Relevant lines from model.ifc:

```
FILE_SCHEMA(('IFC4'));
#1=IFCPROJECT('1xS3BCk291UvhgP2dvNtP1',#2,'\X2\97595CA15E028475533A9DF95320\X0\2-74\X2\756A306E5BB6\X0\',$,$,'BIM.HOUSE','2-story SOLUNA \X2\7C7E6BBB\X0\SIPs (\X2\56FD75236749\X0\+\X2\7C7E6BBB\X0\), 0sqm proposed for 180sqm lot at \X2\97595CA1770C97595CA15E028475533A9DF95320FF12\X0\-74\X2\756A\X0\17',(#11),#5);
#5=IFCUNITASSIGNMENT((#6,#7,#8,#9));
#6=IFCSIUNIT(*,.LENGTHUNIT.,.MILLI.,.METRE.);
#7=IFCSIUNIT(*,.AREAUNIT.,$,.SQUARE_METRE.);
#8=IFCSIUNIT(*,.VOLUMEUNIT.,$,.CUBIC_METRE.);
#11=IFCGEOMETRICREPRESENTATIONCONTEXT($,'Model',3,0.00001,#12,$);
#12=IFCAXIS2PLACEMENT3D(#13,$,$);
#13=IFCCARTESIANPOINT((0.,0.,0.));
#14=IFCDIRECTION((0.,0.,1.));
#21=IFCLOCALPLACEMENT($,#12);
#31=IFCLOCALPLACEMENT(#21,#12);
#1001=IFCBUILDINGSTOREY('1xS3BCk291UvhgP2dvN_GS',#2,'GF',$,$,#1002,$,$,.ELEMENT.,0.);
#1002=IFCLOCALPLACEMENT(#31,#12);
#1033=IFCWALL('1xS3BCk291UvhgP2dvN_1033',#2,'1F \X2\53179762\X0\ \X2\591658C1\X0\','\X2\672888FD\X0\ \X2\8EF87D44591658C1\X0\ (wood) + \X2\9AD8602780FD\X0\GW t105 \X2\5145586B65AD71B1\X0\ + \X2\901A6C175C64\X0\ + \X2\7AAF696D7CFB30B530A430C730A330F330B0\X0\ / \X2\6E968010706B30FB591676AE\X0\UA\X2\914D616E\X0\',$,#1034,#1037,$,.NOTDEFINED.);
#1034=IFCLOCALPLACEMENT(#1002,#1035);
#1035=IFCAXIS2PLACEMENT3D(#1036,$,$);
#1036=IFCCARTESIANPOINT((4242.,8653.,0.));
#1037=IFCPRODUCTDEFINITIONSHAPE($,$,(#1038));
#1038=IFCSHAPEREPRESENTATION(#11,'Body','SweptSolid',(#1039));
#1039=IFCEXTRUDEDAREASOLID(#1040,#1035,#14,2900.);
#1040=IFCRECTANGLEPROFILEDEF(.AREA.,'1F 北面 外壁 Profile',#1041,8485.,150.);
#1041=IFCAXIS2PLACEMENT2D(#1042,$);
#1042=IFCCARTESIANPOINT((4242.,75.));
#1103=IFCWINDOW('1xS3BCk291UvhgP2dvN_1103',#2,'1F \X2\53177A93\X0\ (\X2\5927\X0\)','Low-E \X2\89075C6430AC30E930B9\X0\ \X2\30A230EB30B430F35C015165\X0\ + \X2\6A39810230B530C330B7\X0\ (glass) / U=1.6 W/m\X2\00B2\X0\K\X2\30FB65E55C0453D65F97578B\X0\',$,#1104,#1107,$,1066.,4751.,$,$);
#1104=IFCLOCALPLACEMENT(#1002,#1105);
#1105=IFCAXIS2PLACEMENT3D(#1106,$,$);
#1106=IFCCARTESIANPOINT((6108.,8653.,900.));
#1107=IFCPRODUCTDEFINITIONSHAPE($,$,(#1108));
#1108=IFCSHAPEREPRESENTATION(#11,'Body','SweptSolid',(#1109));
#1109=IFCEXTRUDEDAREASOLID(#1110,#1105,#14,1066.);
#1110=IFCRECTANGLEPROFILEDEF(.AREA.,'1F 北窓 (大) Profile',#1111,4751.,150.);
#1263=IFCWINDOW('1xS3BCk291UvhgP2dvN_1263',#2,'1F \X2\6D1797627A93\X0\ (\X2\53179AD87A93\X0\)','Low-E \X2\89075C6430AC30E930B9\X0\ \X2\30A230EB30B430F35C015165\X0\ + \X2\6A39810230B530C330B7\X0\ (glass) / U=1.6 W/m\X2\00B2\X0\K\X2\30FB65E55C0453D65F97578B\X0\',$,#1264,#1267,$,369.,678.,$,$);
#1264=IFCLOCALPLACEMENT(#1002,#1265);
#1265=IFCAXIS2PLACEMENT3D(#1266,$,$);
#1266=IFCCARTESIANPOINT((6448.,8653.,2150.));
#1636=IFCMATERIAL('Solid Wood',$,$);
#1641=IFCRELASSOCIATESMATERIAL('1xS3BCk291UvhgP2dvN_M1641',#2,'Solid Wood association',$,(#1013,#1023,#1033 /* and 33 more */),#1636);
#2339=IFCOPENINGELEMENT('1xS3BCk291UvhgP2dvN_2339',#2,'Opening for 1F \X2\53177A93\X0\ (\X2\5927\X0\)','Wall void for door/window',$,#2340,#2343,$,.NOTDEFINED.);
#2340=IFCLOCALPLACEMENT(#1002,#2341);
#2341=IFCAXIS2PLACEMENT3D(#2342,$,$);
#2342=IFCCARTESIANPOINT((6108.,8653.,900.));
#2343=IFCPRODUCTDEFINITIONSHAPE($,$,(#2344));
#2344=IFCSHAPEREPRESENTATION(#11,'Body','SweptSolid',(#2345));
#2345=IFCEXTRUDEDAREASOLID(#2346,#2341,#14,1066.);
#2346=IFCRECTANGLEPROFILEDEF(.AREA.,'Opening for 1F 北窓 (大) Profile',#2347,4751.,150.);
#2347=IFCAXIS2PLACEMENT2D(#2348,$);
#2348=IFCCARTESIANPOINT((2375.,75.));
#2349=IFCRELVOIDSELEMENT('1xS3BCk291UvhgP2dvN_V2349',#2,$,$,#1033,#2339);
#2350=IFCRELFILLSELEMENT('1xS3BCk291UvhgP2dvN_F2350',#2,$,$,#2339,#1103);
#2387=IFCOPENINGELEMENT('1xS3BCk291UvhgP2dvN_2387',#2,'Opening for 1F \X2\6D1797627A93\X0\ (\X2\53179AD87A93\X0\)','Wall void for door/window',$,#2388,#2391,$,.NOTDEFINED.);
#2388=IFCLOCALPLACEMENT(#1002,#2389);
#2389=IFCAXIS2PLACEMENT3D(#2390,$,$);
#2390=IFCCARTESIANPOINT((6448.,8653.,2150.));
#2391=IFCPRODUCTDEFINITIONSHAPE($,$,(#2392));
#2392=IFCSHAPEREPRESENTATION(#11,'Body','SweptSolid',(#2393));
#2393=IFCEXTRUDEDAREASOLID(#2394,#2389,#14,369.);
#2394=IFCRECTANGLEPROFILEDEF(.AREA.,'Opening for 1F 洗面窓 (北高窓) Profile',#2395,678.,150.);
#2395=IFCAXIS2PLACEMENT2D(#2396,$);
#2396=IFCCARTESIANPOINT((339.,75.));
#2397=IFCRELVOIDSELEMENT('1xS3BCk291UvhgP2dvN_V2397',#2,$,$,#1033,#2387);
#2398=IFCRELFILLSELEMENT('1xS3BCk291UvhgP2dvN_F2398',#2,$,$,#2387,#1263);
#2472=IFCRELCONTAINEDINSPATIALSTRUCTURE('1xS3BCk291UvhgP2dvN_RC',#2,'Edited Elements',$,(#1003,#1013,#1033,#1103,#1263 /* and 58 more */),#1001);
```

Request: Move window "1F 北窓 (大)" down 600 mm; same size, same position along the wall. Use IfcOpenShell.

```python
import numpy as np
import ifcopenshell
import ifcopenshell.api.geometry
import ifcopenshell.util.placement
import ifcopenshell.util.unit

model = ifcopenshell.open("model.ifc")
unit_scale = ifcopenshell.util.unit.calculate_unit_scale(model)

window = model.by_guid("1xS3BCk291UvhgP2dvN_1103")
opening = window.FillsVoids[0].RelatingOpeningElement
dz = -600.0

shift = np.array([0.0, 0.0, dz])
# The window is not placed relative to its opening, so move both.
for product in (opening, window):
    matrix = ifcopenshell.util.placement.get_local_placement(product.ObjectPlacement)
    matrix[:3, 3] += shift
    ifcopenshell.api.geometry.edit_object_placement(model, product=product, matrix=matrix, is_si=False)

print(f"moved by {dz * unit_scale:+.3f} m")

model.write("model_edited.ifc")
```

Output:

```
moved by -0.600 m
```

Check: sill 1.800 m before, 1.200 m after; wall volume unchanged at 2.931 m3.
